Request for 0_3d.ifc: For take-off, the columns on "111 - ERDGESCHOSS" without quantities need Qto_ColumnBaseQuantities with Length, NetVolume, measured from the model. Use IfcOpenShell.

First a look at what the model holds.

```python
import ifcopenshell
import ifcopenshell.util.element
import ifcopenshell.util.unit

model = ifcopenshell.open("0_3d.ifc")
print(model.schema)
for unit_type in ("LENGTHUNIT", "AREAUNIT", "VOLUMEUNIT"):
    print(unit_type, ifcopenshell.util.unit.calculate_unit_scale(model, unit_type))
storey = next(s for s in model.by_type("IfcBuildingStorey") if s.Name == "111 - ERDGESCHOSS")
columns = [e for e in ifcopenshell.util.element.get_decomposition(storey) if e.is_a("IfcColumn")]
for e in sorted(columns, key=lambda e: e.id()):
    print(e.id(), e.is_a(), e.Name, list(ifcopenshell.util.element.get_psets(e, qtos_only=True)), sep=" | ")
```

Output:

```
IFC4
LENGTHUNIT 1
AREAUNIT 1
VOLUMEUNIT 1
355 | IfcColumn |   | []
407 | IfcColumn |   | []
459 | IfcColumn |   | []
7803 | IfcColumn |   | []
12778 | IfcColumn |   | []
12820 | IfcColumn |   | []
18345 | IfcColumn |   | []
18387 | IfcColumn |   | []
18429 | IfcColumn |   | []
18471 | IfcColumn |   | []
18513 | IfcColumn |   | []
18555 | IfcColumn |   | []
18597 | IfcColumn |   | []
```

```python
import ifcopenshell
import ifcopenshell.api.pset
import ifcopenshell.geom
import ifcopenshell.util.element
import ifcopenshell.util.shape
import ifcopenshell.util.unit

model = ifcopenshell.open("0_3d.ifc")
unit_scale = ifcopenshell.util.unit.calculate_unit_scale(model)
volume_scale = ifcopenshell.util.unit.calculate_unit_scale(model, "VOLUMEUNIT")
settings = ifcopenshell.geom.settings()

storey = next(s for s in model.by_type("IfcBuildingStorey") if s.Name == "111 - ERDGESCHOSS")
columns = [e for e in ifcopenshell.util.element.get_decomposition(storey) if e.is_a("IfcColumn")]

for e in sorted(columns, key=lambda e: e.id()):
    if ifcopenshell.util.element.get_psets(e, qtos_only=True, should_inherit=False):
        continue
    # Geometry comes back in metres, in the element's own axes.
    shape = ifcopenshell.geom.create_shape(settings, e)
    values = {
        "Length": ifcopenshell.util.shape.get_z(shape.geometry) / unit_scale,
        "NetVolume": ifcopenshell.util.shape.get_volume(shape.geometry) / volume_scale,
    }
    qto = ifcopenshell.api.pset.add_qto(model, product=e, name="Qto_ColumnBaseQuantities")
    ifcopenshell.api.pset.edit_qto(model, qto=qto, properties=values)
    print(e.id(), {k: round(v, 3) for k, v in values.items()})

model.write("0_3d_v2.ifc")
```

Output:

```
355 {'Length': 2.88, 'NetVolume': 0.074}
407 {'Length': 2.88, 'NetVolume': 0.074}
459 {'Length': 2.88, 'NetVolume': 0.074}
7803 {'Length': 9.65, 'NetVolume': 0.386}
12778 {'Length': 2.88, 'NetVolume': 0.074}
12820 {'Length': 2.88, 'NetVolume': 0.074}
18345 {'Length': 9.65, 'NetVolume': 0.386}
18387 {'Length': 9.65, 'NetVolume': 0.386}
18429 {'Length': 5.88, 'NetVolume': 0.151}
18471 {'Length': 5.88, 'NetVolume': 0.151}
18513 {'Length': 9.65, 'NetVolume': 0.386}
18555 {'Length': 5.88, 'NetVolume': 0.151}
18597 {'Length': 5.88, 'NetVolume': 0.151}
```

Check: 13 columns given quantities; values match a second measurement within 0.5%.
